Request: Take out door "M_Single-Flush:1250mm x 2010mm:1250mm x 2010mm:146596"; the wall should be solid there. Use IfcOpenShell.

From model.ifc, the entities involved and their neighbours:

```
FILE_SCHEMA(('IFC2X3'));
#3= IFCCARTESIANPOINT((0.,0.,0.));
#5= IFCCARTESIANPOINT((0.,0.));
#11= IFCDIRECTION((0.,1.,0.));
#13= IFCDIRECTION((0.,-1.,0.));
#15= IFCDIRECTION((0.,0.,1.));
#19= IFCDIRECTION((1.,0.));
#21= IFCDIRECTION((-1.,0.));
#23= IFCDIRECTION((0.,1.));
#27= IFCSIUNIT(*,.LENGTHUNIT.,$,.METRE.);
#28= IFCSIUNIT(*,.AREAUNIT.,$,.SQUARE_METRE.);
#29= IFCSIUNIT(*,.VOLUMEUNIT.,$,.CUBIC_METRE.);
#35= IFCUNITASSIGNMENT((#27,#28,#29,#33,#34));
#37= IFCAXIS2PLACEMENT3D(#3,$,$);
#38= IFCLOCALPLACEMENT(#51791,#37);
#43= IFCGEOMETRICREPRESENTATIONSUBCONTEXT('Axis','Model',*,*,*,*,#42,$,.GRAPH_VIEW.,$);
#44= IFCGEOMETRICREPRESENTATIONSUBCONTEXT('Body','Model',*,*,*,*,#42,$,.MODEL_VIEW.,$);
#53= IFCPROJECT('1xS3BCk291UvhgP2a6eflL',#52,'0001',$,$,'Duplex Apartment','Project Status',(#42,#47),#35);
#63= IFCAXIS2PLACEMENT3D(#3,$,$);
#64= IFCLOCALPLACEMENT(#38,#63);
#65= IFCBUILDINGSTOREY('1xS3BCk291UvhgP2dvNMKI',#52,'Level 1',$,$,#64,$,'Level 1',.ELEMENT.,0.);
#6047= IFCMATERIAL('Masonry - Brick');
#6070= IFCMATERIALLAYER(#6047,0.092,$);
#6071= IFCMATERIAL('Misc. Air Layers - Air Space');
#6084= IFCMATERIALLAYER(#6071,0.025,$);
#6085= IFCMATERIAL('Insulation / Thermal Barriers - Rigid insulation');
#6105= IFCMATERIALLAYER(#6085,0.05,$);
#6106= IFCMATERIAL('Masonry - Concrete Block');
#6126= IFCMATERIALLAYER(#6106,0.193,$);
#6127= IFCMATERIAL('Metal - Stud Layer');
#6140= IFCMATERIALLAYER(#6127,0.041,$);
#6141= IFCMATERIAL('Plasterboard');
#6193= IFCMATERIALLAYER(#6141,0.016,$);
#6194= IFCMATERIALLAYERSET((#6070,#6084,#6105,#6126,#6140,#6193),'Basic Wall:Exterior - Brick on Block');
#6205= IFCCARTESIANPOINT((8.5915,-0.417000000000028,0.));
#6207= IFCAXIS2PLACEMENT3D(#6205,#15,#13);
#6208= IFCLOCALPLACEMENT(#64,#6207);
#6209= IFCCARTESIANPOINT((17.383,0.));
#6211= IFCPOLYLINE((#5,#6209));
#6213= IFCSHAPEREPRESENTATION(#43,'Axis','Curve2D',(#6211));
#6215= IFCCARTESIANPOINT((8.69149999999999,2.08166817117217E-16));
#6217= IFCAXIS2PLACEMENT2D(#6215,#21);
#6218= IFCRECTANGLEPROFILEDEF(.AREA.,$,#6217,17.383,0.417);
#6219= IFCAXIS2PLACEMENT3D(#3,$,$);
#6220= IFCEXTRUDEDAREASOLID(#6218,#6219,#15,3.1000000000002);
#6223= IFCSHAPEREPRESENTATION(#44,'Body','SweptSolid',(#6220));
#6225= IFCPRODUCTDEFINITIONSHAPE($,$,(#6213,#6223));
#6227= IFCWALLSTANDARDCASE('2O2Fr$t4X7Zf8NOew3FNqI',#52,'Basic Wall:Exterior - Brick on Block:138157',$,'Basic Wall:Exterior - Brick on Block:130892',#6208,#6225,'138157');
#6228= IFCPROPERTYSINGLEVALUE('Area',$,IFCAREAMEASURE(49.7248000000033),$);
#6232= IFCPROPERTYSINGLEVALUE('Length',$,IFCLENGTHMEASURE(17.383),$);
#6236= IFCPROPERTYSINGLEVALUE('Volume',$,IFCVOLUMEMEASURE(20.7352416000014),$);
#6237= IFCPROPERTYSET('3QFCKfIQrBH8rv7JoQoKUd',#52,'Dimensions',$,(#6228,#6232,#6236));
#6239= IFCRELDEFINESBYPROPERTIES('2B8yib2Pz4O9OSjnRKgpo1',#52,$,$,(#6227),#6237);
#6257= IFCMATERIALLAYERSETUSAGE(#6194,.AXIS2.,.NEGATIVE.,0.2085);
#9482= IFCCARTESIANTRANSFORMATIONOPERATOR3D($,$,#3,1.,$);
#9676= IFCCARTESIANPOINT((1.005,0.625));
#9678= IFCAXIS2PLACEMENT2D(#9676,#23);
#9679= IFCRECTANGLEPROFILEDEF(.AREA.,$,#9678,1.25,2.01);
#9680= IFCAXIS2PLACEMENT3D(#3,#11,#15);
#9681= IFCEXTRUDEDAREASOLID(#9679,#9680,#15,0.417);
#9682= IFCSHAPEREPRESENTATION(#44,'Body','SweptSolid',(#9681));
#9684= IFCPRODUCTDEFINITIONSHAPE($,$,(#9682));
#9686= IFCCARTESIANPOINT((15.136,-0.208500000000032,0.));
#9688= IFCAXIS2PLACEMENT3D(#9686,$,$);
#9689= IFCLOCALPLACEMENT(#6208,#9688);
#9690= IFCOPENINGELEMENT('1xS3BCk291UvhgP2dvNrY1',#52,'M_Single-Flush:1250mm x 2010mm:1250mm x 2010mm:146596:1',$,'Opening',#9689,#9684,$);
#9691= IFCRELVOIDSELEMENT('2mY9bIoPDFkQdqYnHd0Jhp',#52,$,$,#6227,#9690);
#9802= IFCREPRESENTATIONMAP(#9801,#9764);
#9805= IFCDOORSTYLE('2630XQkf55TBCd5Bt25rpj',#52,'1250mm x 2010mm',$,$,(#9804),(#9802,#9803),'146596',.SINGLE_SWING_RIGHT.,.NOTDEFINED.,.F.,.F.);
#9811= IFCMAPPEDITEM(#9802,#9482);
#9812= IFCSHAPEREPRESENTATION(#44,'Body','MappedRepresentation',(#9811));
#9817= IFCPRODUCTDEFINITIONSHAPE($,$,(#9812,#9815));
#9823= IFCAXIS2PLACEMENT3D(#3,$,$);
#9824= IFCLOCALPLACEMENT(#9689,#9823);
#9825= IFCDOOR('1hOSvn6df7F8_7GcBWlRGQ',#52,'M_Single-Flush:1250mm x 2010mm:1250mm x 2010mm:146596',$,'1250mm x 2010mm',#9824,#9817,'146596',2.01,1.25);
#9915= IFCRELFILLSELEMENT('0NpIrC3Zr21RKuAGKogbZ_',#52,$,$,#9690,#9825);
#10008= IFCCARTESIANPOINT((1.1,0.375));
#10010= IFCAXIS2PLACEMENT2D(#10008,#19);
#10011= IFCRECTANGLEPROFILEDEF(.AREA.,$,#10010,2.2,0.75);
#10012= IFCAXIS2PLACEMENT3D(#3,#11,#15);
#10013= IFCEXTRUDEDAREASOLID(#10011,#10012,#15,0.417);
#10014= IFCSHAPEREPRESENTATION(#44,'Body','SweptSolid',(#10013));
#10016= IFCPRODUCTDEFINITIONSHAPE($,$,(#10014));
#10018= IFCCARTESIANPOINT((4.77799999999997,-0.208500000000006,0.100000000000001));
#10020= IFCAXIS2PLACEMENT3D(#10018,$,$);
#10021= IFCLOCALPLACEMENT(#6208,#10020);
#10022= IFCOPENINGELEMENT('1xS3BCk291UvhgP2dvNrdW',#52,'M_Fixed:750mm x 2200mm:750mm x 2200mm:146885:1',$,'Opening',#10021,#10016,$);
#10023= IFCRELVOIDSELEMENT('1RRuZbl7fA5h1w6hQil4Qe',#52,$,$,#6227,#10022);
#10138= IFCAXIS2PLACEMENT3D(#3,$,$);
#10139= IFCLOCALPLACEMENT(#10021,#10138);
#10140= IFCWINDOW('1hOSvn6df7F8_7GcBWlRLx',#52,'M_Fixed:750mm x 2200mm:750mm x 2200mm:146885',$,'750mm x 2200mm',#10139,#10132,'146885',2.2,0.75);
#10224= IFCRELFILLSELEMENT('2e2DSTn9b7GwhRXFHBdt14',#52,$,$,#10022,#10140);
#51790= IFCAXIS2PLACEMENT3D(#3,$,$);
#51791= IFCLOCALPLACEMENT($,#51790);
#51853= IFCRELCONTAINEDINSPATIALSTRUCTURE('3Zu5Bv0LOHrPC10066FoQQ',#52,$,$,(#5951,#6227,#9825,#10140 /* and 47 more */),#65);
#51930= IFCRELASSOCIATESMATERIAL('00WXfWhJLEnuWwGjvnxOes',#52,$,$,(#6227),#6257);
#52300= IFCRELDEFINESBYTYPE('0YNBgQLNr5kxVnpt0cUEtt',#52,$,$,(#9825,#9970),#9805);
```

```python
import ifcopenshell
import ifcopenshell.api.feature
import ifcopenshell.api.pset
import ifcopenshell.api.root
import ifcopenshell.geom
import ifcopenshell.util.element
import ifcopenshell.util.shape
import ifcopenshell.util.unit

model = ifcopenshell.open("model.ifc")
area_scale = ifcopenshell.util.unit.calculate_unit_scale(model, "AREAUNIT")
volume_scale = ifcopenshell.util.unit.calculate_unit_scale(model, "VOLUMEUNIT")
settings = ifcopenshell.geom.settings()


def volume(element):
    """Net volume in cubic metres, openings subtracted."""
    shape = ifcopenshell.geom.create_shape(settings, element)
    return ifcopenshell.util.shape.get_volume(shape.geometry)


door = model.by_guid("1hOSvn6df7F8_7GcBWlRGQ")
opening = door.FillsVoids[0].RelatingOpeningElement
wall = opening.VoidsElements[0].RelatingBuildingElement
before = volume(wall)

ifcopenshell.api.root.remove_product(model, product=door)
ifcopenshell.api.feature.remove_feature(model, feature=opening)

after = volume(wall)
thickness = 0.417  # wall thickness in metres

# Update the wall's stored quantities.
pset = model.by_id(ifcopenshell.util.element.get_pset(wall, "Dimensions", should_inherit=False)["id"])
ifcopenshell.api.pset.edit_pset(model, pset=pset, properties={
    "Area": model.create_entity("IfcAreaMeasure", after / thickness / area_scale),
    "Volume": model.create_entity("IfcVolumeMeasure", after / volume_scale),
})

print(f"wall volume {before:.3f} -> {after:.3f} m3")

model.write("model_updated.ifc")
```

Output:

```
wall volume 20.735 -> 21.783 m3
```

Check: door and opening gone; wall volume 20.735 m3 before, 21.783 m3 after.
